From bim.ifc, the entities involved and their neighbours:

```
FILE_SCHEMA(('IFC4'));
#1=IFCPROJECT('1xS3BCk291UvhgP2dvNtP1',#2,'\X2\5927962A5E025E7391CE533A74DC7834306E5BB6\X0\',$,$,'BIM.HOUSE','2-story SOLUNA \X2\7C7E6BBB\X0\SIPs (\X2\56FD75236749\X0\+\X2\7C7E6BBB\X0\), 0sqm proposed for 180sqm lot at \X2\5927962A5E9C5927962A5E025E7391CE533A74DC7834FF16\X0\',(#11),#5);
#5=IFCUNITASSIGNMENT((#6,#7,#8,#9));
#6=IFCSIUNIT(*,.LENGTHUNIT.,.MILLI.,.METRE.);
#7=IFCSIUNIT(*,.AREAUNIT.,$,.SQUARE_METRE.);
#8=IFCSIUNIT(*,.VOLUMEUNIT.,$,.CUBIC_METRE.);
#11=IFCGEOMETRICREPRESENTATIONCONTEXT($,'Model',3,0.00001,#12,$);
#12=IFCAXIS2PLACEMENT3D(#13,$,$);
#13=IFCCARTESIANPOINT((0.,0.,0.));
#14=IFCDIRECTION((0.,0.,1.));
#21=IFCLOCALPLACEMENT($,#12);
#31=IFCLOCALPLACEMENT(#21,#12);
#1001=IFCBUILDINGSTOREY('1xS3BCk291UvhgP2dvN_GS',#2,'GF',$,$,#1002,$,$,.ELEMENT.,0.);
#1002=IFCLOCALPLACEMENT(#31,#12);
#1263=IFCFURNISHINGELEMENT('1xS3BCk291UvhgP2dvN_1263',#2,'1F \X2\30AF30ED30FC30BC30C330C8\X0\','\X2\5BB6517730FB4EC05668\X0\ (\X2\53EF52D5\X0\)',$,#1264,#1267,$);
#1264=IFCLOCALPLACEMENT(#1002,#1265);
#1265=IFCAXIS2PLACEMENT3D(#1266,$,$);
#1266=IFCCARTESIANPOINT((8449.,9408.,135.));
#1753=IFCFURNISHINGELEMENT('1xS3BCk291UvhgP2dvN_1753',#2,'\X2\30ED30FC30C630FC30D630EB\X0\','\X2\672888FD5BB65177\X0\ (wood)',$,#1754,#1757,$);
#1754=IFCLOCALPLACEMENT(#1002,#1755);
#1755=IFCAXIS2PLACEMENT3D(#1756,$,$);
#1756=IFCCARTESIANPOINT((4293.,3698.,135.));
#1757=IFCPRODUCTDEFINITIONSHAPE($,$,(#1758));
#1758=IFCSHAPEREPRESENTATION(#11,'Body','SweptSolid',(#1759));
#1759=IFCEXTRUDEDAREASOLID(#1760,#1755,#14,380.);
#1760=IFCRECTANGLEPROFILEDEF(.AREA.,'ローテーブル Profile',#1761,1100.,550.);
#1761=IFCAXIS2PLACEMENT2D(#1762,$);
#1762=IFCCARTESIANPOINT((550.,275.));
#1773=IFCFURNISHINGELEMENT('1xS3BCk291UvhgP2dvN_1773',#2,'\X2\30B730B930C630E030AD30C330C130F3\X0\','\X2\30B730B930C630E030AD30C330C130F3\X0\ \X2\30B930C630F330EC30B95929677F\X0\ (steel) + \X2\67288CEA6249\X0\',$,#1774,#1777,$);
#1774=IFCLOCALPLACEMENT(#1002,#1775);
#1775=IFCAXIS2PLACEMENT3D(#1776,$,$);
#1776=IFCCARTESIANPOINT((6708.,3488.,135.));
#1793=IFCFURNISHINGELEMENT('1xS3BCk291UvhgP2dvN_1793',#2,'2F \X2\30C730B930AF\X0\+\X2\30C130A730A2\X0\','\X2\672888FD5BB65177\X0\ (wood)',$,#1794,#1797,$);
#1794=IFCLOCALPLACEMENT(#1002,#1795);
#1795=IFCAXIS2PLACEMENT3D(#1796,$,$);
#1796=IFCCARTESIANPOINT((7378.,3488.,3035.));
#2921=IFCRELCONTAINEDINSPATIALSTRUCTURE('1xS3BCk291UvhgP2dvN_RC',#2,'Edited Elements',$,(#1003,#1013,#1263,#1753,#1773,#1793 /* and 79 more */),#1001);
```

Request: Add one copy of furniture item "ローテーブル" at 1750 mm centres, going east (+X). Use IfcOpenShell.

```python
import numpy as np
import ifcopenshell
import ifcopenshell.api.geometry
import ifcopenshell.api.root
import ifcopenshell.util.element
import ifcopenshell.util.placement
import ifcopenshell.util.unit

model = ifcopenshell.open("bim.ifc")
unit_scale = ifcopenshell.util.unit.calculate_unit_scale(model)


def reuse_history(source, copy):
    """copy_class also copies each property set's owner history, people and application; keep the originals."""
    for rel in copy.IsDefinedBy:
        if rel.is_a("IfcRelDefinesByProperties") and (history := rel.RelatingPropertyDefinition.OwnerHistory):
            rel.RelatingPropertyDefinition.OwnerHistory = source.OwnerHistory
            ifcopenshell.util.element.remove_deep2(model, history)


source = model.by_guid("1xS3BCk291UvhgP2dvN_1753")
base = ifcopenshell.util.placement.get_local_placement(source.ObjectPlacement)
step = np.array([1.0, 0.0, 0.0]) * 1.75 / unit_scale

for i in range(1, 2):
    copy = ifcopenshell.api.root.copy_class(model, product=source)
    copy.Representation = ifcopenshell.util.element.copy_deep(
        model, source.Representation, exclude=["IfcGeometricRepresentationContext", "IfcRepresentationMap"]
    )
    reuse_history(source, copy)
    matrix = base.copy()
    matrix[:3, 3] += i * step
    print("added at", matrix[:3, 3].round(3) + 0.0)
    ifcopenshell.api.geometry.edit_object_placement(model, product=copy, matrix=matrix, is_si=False)

model.write("bim-out.ifc")
```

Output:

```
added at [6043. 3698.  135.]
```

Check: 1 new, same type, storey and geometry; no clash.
